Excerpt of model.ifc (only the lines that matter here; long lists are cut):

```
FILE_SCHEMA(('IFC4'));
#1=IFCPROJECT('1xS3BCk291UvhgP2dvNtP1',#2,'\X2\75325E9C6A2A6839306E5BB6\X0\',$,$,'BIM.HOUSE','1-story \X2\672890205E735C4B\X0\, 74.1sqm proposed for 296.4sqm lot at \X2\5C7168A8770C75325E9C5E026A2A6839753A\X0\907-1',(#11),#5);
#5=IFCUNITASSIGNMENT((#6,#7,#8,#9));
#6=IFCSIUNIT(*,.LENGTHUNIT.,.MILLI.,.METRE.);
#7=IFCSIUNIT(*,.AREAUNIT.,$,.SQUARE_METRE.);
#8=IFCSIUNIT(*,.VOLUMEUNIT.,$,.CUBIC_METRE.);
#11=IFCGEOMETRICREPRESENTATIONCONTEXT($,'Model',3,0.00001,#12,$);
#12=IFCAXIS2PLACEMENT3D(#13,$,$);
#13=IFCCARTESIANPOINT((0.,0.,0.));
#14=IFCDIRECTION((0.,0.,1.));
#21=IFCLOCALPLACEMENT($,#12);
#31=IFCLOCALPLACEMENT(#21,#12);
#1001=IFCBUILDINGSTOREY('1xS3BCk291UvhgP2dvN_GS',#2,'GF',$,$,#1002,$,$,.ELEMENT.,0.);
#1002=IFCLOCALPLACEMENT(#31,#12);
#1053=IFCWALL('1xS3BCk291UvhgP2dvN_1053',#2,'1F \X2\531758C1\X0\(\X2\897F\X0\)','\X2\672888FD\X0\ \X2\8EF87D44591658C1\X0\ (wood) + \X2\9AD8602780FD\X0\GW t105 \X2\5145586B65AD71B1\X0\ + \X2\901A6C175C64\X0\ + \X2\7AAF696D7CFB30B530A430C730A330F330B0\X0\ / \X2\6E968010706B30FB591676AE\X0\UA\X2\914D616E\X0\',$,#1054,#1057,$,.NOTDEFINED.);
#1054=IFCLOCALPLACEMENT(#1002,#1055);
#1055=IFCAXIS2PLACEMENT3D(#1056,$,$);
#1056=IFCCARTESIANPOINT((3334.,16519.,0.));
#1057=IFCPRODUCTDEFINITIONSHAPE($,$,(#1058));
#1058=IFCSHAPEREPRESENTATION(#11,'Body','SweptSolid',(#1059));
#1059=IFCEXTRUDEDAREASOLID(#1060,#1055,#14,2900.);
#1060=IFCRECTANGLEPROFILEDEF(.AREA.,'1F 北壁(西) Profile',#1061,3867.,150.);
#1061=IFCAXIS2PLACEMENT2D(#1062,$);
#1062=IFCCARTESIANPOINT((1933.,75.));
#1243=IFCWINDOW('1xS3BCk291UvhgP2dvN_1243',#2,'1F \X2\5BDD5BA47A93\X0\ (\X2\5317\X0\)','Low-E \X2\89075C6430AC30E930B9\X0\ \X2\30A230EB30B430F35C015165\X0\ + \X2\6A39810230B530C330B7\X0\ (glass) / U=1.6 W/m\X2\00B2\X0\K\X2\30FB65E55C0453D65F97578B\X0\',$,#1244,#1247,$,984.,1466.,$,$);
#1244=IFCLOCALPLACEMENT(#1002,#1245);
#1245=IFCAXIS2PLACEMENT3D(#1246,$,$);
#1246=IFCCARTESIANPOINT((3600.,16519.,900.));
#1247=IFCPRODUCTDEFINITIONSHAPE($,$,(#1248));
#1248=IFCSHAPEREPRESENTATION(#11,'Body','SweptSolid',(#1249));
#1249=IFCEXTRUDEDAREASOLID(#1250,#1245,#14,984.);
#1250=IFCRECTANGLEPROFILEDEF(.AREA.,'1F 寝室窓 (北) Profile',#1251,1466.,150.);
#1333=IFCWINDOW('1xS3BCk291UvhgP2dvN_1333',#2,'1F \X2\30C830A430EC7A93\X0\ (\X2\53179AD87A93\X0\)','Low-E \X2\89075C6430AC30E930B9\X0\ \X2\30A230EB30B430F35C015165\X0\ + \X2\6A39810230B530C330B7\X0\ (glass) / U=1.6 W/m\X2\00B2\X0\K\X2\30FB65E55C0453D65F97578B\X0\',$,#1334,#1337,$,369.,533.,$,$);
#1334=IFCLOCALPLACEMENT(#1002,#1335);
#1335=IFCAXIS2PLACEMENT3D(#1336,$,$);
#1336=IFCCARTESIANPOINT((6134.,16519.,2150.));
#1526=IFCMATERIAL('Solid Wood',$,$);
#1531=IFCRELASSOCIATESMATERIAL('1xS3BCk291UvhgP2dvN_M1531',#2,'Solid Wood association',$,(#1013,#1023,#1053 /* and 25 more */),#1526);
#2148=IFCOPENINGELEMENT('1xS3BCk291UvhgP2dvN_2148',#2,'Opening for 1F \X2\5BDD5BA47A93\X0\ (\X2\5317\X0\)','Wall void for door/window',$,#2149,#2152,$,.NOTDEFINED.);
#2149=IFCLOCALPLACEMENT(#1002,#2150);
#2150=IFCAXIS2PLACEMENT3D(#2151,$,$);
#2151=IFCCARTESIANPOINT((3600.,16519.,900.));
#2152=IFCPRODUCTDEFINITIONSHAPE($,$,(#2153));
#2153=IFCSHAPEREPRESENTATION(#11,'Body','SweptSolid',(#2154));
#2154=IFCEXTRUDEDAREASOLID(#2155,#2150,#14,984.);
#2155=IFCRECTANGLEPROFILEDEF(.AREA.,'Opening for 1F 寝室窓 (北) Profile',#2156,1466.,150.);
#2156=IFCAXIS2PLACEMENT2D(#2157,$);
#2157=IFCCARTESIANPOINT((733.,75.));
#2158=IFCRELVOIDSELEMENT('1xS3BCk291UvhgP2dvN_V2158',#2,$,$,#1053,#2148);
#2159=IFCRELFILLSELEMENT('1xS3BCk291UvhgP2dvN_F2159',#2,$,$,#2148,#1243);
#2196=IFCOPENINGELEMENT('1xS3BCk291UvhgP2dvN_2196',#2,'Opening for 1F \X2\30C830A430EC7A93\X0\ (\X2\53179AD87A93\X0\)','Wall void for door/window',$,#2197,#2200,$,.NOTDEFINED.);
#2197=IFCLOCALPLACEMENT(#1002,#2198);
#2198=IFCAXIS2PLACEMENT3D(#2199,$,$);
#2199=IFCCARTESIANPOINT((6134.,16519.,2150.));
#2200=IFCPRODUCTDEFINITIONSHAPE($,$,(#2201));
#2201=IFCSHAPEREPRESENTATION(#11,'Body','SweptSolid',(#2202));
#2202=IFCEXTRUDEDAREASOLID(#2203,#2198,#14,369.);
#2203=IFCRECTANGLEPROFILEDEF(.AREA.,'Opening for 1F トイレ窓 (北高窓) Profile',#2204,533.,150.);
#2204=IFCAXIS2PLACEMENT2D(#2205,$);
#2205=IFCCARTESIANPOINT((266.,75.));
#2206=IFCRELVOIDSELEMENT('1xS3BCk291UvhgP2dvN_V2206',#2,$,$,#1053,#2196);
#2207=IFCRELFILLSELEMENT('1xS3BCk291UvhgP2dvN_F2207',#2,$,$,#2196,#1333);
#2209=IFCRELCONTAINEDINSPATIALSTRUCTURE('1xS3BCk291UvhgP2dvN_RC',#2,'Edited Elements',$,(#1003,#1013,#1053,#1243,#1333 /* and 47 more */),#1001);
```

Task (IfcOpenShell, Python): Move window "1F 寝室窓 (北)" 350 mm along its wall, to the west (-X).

```python
import ifcopenshell
import ifcopenshell.api.geometry
import ifcopenshell.util.placement
import ifcopenshell.util.unit

model = ifcopenshell.open("model.ifc")
unit_scale = ifcopenshell.util.unit.calculate_unit_scale(model)

window = model.by_guid("1xS3BCk291UvhgP2dvN_1243")
opening = window.FillsVoids[0].RelatingOpeningElement
wall = opening.VoidsElements[0].RelatingBuildingElement

wall_matrix = ifcopenshell.util.placement.get_local_placement(wall.ObjectPlacement)
shift = wall_matrix[:3, 0] * -0.35 / unit_scale
before = ifcopenshell.util.placement.get_local_placement(window.ObjectPlacement)[:3, 3].copy()

# The window is not placed relative to its opening, so move both.
for product in (opening, window):
    matrix = ifcopenshell.util.placement.get_local_placement(product.ObjectPlacement)
    matrix[:3, 3] += shift
    ifcopenshell.api.geometry.edit_object_placement(model, product=product, matrix=matrix, is_si=False)

after = ifcopenshell.util.placement.get_local_placement(window.ObjectPlacement)[:3, 3]
print("window moved by", (after - before).round(3) + 0.0)

model.write("model_rev.ifc")
```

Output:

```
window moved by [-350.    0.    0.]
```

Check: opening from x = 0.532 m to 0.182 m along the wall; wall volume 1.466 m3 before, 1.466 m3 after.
